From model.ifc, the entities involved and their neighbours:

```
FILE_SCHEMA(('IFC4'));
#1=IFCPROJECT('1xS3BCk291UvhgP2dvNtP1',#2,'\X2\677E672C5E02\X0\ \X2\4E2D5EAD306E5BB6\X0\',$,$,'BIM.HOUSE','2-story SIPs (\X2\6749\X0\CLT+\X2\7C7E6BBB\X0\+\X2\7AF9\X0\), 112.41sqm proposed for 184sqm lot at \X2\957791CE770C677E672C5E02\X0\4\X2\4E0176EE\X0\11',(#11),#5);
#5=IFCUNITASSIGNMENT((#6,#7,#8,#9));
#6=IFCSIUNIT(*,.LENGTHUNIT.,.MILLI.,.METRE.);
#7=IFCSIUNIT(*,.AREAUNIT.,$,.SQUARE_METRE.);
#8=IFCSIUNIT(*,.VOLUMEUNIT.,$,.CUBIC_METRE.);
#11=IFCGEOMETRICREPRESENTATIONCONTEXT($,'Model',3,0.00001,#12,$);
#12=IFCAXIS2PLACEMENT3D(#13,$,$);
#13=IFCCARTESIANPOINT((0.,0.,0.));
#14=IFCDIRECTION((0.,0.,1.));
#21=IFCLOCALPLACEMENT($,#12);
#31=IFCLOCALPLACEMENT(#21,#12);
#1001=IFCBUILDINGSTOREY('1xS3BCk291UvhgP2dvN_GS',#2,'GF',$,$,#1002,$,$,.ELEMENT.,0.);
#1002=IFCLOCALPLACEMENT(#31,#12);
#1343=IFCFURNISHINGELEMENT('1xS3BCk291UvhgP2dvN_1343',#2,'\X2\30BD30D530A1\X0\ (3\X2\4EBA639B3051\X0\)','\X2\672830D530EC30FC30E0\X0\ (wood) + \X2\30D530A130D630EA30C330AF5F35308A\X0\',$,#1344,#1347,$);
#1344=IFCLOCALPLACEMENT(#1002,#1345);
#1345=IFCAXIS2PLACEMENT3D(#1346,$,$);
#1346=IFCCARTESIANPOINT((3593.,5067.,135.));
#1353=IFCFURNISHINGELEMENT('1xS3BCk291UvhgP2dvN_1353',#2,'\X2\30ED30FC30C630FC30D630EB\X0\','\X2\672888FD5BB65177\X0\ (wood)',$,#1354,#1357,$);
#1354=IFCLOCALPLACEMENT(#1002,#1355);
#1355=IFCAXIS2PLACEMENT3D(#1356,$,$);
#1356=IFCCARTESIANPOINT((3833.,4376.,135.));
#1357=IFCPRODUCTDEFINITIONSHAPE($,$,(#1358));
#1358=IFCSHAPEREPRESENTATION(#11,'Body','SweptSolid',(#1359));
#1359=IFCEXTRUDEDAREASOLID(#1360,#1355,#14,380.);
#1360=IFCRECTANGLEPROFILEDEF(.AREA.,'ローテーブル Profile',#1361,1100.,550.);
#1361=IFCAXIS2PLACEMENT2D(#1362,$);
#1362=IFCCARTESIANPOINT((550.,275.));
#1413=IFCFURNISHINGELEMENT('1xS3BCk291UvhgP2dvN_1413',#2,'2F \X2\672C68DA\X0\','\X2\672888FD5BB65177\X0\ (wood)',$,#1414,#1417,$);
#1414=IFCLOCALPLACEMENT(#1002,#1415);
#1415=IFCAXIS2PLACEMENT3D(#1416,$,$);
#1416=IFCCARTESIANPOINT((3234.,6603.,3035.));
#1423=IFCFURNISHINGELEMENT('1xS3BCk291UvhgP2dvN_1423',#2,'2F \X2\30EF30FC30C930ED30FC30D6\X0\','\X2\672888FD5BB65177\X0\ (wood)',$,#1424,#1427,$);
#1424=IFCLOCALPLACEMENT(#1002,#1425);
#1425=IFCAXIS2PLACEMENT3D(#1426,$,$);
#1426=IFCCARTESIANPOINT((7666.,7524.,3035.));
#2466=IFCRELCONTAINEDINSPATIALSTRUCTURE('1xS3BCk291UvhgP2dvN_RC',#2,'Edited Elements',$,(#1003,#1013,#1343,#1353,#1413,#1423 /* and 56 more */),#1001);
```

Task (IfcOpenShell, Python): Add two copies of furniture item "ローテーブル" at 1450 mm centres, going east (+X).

```python
import numpy as np
import ifcopenshell
import ifcopenshell.api.geometry
import ifcopenshell.api.root
import ifcopenshell.util.element
import ifcopenshell.util.placement
import ifcopenshell.util.unit

model = ifcopenshell.open("model.ifc")
unit_scale = ifcopenshell.util.unit.calculate_unit_scale(model)


def reuse_history(source, copy):
    """copy_class also copies each property set's owner history, people and application; keep the originals."""
    for rel in copy.IsDefinedBy:
        if rel.is_a("IfcRelDefinesByProperties") and (history := rel.RelatingPropertyDefinition.OwnerHistory):
            rel.RelatingPropertyDefinition.OwnerHistory = source.OwnerHistory
            ifcopenshell.util.element.remove_deep2(model, history)


source = model.by_id(1353)
base = ifcopenshell.util.placement.get_local_placement(source.ObjectPlacement)
step = np.array([1.0, 0.0, 0.0]) * 1.45 / unit_scale

for i in range(1, 3):
    copy = ifcopenshell.api.root.copy_class(model, product=source)
    copy.Representation = ifcopenshell.util.element.copy_deep(
        model, source.Representation, exclude=["IfcGeometricRepresentationContext", "IfcRepresentationMap"]
    )
    reuse_history(source, copy)
    matrix = base.copy()
    matrix[:3, 3] += i * step
    print("added at", matrix[:3, 3].round(3) + 0.0)
    ifcopenshell.api.geometry.edit_object_placement(model, product=copy, matrix=matrix, is_si=False)

model.write("model-out.ifc")
```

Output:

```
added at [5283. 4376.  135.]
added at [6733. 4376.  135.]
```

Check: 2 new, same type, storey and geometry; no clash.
